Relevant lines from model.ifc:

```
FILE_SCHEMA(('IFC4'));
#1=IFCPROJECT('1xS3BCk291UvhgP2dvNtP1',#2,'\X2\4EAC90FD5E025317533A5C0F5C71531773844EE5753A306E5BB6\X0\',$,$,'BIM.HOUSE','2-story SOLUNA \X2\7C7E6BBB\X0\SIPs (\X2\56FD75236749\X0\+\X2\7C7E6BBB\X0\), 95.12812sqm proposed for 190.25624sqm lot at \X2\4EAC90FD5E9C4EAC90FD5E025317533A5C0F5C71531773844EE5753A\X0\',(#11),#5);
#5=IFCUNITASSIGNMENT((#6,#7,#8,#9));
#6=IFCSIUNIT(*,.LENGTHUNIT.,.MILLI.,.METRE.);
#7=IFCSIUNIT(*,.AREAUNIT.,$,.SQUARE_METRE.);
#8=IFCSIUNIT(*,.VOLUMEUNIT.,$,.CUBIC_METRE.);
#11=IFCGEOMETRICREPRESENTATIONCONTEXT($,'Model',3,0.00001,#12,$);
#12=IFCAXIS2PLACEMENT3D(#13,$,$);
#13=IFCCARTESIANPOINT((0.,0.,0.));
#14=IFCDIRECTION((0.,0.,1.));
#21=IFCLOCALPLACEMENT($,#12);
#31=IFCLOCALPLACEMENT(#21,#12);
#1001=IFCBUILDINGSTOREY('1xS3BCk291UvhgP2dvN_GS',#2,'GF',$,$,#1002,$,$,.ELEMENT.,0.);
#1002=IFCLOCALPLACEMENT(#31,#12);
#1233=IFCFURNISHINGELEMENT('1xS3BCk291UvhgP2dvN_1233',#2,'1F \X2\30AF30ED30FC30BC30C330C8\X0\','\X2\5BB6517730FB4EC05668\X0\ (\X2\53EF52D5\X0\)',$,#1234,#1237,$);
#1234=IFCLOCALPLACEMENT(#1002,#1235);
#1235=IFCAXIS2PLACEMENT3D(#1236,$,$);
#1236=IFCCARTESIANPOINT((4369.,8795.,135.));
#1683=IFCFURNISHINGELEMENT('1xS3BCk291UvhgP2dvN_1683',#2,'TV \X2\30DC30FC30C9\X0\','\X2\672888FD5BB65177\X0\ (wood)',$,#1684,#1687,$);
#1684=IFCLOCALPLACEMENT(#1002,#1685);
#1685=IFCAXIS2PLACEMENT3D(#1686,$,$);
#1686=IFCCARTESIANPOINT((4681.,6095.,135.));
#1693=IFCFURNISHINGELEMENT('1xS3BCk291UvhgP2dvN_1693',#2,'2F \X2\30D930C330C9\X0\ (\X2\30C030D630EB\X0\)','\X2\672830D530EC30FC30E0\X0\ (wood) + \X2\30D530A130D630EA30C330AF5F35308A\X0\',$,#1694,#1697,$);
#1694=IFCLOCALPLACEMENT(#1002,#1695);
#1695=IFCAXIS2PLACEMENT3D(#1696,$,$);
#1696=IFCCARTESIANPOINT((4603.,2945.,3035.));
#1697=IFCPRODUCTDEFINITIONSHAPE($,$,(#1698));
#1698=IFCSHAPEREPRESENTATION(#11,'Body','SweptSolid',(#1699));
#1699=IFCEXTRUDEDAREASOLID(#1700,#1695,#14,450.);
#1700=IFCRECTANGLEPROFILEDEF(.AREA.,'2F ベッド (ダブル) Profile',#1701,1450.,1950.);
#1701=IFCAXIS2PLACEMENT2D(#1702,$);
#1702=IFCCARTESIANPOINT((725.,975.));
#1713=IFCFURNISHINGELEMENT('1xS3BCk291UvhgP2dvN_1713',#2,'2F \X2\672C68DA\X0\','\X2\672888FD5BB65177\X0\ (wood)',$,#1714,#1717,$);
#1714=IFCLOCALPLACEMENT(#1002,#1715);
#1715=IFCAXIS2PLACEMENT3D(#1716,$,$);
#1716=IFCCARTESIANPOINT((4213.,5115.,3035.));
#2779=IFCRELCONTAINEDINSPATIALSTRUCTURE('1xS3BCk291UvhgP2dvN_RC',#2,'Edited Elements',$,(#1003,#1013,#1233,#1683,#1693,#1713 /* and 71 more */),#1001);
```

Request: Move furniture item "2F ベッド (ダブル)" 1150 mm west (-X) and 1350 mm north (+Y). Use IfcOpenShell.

```python
import ifcopenshell
import ifcopenshell.api.geometry
import ifcopenshell.util.placement

model = ifcopenshell.open("model.ifc")

item = model.by_guid("1xS3BCk291UvhgP2dvN_1693")
matrix = ifcopenshell.util.placement.get_local_placement(item.ObjectPlacement)
matrix[0, 3] -= 1150.0
matrix[1, 3] += 1350.0
ifcopenshell.api.geometry.edit_object_placement(model, product=item, matrix=matrix, is_si=False)

print(ifcopenshell.util.placement.get_local_placement(item.ObjectPlacement).round(3) + 0.0)

model.write("model_edited.ifc")
```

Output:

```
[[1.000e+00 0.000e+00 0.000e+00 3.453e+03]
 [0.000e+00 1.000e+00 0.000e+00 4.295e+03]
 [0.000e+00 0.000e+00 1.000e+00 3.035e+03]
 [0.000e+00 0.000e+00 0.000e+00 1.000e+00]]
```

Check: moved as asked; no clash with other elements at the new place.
